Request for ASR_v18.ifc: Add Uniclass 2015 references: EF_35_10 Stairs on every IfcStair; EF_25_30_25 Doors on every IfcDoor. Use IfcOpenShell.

First a look at what the model holds.

```python
import ifcopenshell

model = ifcopenshell.open("ASR_v18.ifc")
print(model.schema)
print("classifications:", [c.Name for c in model.by_type("IfcClassification")])
for ifc_class in ("IfcDoor", "IfcRoof", "IfcStair", "IfcWall", "IfcWindow"):
    print(ifc_class, len(model.by_type(ifc_class)))
```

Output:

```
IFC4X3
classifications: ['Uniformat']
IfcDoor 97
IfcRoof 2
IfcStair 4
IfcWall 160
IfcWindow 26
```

```python
import ifcopenshell
import ifcopenshell.api.classification

model = ifcopenshell.open("ASR_v18.ifc")

system = ifcopenshell.api.classification.add_classification(model, classification="Uniclass 2015")

codes = {
    "IfcStair": ("EF_35_10", "Stairs"),
    "IfcDoor": ("EF_25_30_25", "Doors"),
}
for ifc_class, (code, name) in codes.items():
    products = model.by_type(ifc_class)
    ifcopenshell.api.classification.add_reference(
        model, products=products, classification=system, identification=code, name=name
    )
    print(code, len(products))

model.write("ASR_v18_updated.ifc")
```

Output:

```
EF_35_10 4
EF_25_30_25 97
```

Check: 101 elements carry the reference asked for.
